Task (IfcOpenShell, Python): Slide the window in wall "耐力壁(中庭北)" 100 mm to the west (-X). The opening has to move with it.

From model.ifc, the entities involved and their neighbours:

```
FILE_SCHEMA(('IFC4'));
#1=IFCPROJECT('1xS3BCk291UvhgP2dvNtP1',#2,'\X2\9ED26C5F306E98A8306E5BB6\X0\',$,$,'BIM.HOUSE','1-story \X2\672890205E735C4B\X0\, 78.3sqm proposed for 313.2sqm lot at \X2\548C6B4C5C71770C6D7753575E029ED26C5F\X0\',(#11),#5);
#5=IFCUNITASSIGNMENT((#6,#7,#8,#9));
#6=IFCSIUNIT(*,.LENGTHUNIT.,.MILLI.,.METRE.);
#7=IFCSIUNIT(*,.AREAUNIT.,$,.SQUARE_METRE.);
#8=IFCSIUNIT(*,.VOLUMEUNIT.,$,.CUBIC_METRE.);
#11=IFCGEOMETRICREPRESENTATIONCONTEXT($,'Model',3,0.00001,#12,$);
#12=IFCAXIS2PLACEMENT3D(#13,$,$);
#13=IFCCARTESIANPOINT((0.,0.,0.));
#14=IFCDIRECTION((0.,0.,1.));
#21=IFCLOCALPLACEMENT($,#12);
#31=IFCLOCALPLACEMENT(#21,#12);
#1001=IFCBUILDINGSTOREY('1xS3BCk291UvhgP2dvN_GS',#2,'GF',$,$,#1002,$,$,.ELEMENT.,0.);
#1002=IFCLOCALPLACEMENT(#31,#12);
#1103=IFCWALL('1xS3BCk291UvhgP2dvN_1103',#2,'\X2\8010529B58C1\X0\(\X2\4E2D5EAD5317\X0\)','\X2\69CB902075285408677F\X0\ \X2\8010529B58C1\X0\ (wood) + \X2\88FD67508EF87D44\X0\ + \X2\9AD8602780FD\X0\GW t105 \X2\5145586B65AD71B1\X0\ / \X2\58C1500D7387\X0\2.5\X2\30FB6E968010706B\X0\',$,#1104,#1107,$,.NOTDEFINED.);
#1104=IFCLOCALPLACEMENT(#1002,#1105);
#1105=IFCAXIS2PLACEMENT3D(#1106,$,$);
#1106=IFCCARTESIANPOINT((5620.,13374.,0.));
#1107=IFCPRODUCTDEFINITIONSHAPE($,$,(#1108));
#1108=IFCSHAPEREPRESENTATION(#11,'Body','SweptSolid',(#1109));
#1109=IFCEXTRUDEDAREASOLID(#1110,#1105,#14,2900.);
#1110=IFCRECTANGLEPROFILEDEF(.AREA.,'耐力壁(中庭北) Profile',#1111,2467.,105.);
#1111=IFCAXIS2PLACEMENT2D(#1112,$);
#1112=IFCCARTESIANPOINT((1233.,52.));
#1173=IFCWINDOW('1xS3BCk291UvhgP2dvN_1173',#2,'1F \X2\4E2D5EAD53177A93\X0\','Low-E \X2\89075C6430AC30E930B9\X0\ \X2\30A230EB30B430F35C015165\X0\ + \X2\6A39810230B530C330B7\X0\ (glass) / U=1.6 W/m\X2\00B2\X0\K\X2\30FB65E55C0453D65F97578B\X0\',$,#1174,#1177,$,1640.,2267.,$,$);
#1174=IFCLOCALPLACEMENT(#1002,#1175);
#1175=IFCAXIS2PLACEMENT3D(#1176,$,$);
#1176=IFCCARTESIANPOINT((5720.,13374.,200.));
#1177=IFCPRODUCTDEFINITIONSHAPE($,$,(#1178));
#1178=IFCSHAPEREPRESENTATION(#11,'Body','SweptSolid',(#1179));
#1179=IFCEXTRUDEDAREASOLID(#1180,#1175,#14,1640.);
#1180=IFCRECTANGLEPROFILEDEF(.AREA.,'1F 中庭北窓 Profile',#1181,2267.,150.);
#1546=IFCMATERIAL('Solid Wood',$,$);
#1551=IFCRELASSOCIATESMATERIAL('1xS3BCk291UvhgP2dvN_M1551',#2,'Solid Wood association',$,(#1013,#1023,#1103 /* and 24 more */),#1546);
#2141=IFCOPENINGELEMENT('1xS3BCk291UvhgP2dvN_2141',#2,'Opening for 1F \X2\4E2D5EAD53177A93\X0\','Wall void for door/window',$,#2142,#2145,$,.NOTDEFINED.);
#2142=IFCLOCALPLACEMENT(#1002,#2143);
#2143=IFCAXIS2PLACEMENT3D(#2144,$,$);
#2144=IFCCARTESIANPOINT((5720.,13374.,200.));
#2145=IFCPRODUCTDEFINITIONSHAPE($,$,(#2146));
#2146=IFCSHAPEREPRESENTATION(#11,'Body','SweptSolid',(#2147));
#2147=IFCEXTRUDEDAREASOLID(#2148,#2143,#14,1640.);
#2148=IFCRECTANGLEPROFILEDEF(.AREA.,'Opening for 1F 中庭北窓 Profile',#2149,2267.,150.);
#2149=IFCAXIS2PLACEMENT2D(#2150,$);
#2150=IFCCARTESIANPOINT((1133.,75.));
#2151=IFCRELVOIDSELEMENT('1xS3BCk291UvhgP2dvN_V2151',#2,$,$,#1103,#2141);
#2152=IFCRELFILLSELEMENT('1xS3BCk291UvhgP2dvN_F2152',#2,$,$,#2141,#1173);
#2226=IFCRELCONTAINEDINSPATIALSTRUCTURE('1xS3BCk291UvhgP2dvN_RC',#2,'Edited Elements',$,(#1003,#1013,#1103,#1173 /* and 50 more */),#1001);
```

```python
import ifcopenshell
import ifcopenshell.api.geometry
import ifcopenshell.util.placement

model = ifcopenshell.open("model.ifc")

window = model.by_guid("1xS3BCk291UvhgP2dvN_1173")
opening = window.FillsVoids[0].RelatingOpeningElement
wall = opening.VoidsElements[0].RelatingBuildingElement

wall_matrix = ifcopenshell.util.placement.get_local_placement(wall.ObjectPlacement)
shift = wall_matrix[:3, 0] * -100.0
before = ifcopenshell.util.placement.get_local_placement(window.ObjectPlacement)[:3, 3].copy()

# The window is not placed relative to its opening, so move both.
for product in (opening, window):
    matrix = ifcopenshell.util.placement.get_local_placement(product.ObjectPlacement)
    matrix[:3, 3] += shift
    ifcopenshell.api.geometry.edit_object_placement(model, product=product, matrix=matrix, is_si=False)

after = ifcopenshell.util.placement.get_local_placement(window.ObjectPlacement)[:3, 3]
print("window moved by", (after - before).round(3) + 0.0)

model.write("model-out.ifc")
```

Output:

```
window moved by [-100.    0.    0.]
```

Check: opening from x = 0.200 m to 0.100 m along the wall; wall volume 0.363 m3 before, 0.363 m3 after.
